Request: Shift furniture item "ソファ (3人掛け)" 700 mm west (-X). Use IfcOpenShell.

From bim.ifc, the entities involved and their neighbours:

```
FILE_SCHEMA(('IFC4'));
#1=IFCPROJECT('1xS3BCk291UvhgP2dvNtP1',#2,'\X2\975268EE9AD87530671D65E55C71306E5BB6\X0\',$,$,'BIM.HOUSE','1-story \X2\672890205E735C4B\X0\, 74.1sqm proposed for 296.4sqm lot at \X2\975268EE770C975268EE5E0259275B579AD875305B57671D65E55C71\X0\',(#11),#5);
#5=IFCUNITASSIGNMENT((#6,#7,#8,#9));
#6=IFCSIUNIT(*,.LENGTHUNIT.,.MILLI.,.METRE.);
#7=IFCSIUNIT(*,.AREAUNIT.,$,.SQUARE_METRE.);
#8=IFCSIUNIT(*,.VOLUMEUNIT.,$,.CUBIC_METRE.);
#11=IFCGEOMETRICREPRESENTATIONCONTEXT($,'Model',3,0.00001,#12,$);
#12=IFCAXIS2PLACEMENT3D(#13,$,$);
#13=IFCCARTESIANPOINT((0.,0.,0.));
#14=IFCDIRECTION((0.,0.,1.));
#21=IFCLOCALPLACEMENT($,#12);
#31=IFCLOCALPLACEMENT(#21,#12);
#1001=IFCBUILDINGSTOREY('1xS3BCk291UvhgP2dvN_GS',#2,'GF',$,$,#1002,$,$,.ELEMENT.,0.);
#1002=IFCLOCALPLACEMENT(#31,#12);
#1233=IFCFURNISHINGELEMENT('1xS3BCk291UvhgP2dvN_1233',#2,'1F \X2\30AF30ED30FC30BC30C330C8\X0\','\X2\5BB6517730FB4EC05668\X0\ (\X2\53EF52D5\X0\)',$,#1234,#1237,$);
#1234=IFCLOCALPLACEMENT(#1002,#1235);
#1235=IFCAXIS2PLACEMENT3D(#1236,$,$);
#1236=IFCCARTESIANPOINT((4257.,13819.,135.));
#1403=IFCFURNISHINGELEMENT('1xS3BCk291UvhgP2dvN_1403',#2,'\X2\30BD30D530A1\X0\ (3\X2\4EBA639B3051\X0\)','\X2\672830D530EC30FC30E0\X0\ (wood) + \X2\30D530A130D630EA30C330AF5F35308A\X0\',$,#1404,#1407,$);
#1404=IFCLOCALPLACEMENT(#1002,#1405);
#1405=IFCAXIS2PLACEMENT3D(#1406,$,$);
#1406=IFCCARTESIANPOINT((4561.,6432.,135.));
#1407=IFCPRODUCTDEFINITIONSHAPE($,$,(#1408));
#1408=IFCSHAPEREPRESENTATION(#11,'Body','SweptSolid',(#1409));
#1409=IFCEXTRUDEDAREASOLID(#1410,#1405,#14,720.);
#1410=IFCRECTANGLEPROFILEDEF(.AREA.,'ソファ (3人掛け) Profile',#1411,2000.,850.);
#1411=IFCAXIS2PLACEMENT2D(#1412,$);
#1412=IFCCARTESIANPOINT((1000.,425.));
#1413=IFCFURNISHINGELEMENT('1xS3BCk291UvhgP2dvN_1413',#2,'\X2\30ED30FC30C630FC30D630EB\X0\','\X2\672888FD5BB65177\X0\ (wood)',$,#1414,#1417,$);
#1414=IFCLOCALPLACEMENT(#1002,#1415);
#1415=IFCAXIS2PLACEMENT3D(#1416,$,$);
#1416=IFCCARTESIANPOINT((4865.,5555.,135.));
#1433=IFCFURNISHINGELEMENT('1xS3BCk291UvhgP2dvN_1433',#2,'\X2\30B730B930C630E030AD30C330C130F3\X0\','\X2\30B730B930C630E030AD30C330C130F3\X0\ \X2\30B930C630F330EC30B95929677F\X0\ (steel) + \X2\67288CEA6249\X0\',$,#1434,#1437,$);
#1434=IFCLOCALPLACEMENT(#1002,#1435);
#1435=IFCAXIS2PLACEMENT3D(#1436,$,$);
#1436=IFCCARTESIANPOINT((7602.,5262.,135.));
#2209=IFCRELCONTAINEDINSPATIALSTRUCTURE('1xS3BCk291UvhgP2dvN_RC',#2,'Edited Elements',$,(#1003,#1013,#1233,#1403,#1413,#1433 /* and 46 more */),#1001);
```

```python
import ifcopenshell
import ifcopenshell.api.geometry
import ifcopenshell.util.placement

model = ifcopenshell.open("bim.ifc")

item = model.by_guid("1xS3BCk291UvhgP2dvN_1403")
matrix = ifcopenshell.util.placement.get_local_placement(item.ObjectPlacement)
matrix[0, 3] -= 700.0
ifcopenshell.api.geometry.edit_object_placement(model, product=item, matrix=matrix, is_si=False)

print(ifcopenshell.util.placement.get_local_placement(item.ObjectPlacement).round(3) + 0.0)

model.write("bim_edited.ifc")
```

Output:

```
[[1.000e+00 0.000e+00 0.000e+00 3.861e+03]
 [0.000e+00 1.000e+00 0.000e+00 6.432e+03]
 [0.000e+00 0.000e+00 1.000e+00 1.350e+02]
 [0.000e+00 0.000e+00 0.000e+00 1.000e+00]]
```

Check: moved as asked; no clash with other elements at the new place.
